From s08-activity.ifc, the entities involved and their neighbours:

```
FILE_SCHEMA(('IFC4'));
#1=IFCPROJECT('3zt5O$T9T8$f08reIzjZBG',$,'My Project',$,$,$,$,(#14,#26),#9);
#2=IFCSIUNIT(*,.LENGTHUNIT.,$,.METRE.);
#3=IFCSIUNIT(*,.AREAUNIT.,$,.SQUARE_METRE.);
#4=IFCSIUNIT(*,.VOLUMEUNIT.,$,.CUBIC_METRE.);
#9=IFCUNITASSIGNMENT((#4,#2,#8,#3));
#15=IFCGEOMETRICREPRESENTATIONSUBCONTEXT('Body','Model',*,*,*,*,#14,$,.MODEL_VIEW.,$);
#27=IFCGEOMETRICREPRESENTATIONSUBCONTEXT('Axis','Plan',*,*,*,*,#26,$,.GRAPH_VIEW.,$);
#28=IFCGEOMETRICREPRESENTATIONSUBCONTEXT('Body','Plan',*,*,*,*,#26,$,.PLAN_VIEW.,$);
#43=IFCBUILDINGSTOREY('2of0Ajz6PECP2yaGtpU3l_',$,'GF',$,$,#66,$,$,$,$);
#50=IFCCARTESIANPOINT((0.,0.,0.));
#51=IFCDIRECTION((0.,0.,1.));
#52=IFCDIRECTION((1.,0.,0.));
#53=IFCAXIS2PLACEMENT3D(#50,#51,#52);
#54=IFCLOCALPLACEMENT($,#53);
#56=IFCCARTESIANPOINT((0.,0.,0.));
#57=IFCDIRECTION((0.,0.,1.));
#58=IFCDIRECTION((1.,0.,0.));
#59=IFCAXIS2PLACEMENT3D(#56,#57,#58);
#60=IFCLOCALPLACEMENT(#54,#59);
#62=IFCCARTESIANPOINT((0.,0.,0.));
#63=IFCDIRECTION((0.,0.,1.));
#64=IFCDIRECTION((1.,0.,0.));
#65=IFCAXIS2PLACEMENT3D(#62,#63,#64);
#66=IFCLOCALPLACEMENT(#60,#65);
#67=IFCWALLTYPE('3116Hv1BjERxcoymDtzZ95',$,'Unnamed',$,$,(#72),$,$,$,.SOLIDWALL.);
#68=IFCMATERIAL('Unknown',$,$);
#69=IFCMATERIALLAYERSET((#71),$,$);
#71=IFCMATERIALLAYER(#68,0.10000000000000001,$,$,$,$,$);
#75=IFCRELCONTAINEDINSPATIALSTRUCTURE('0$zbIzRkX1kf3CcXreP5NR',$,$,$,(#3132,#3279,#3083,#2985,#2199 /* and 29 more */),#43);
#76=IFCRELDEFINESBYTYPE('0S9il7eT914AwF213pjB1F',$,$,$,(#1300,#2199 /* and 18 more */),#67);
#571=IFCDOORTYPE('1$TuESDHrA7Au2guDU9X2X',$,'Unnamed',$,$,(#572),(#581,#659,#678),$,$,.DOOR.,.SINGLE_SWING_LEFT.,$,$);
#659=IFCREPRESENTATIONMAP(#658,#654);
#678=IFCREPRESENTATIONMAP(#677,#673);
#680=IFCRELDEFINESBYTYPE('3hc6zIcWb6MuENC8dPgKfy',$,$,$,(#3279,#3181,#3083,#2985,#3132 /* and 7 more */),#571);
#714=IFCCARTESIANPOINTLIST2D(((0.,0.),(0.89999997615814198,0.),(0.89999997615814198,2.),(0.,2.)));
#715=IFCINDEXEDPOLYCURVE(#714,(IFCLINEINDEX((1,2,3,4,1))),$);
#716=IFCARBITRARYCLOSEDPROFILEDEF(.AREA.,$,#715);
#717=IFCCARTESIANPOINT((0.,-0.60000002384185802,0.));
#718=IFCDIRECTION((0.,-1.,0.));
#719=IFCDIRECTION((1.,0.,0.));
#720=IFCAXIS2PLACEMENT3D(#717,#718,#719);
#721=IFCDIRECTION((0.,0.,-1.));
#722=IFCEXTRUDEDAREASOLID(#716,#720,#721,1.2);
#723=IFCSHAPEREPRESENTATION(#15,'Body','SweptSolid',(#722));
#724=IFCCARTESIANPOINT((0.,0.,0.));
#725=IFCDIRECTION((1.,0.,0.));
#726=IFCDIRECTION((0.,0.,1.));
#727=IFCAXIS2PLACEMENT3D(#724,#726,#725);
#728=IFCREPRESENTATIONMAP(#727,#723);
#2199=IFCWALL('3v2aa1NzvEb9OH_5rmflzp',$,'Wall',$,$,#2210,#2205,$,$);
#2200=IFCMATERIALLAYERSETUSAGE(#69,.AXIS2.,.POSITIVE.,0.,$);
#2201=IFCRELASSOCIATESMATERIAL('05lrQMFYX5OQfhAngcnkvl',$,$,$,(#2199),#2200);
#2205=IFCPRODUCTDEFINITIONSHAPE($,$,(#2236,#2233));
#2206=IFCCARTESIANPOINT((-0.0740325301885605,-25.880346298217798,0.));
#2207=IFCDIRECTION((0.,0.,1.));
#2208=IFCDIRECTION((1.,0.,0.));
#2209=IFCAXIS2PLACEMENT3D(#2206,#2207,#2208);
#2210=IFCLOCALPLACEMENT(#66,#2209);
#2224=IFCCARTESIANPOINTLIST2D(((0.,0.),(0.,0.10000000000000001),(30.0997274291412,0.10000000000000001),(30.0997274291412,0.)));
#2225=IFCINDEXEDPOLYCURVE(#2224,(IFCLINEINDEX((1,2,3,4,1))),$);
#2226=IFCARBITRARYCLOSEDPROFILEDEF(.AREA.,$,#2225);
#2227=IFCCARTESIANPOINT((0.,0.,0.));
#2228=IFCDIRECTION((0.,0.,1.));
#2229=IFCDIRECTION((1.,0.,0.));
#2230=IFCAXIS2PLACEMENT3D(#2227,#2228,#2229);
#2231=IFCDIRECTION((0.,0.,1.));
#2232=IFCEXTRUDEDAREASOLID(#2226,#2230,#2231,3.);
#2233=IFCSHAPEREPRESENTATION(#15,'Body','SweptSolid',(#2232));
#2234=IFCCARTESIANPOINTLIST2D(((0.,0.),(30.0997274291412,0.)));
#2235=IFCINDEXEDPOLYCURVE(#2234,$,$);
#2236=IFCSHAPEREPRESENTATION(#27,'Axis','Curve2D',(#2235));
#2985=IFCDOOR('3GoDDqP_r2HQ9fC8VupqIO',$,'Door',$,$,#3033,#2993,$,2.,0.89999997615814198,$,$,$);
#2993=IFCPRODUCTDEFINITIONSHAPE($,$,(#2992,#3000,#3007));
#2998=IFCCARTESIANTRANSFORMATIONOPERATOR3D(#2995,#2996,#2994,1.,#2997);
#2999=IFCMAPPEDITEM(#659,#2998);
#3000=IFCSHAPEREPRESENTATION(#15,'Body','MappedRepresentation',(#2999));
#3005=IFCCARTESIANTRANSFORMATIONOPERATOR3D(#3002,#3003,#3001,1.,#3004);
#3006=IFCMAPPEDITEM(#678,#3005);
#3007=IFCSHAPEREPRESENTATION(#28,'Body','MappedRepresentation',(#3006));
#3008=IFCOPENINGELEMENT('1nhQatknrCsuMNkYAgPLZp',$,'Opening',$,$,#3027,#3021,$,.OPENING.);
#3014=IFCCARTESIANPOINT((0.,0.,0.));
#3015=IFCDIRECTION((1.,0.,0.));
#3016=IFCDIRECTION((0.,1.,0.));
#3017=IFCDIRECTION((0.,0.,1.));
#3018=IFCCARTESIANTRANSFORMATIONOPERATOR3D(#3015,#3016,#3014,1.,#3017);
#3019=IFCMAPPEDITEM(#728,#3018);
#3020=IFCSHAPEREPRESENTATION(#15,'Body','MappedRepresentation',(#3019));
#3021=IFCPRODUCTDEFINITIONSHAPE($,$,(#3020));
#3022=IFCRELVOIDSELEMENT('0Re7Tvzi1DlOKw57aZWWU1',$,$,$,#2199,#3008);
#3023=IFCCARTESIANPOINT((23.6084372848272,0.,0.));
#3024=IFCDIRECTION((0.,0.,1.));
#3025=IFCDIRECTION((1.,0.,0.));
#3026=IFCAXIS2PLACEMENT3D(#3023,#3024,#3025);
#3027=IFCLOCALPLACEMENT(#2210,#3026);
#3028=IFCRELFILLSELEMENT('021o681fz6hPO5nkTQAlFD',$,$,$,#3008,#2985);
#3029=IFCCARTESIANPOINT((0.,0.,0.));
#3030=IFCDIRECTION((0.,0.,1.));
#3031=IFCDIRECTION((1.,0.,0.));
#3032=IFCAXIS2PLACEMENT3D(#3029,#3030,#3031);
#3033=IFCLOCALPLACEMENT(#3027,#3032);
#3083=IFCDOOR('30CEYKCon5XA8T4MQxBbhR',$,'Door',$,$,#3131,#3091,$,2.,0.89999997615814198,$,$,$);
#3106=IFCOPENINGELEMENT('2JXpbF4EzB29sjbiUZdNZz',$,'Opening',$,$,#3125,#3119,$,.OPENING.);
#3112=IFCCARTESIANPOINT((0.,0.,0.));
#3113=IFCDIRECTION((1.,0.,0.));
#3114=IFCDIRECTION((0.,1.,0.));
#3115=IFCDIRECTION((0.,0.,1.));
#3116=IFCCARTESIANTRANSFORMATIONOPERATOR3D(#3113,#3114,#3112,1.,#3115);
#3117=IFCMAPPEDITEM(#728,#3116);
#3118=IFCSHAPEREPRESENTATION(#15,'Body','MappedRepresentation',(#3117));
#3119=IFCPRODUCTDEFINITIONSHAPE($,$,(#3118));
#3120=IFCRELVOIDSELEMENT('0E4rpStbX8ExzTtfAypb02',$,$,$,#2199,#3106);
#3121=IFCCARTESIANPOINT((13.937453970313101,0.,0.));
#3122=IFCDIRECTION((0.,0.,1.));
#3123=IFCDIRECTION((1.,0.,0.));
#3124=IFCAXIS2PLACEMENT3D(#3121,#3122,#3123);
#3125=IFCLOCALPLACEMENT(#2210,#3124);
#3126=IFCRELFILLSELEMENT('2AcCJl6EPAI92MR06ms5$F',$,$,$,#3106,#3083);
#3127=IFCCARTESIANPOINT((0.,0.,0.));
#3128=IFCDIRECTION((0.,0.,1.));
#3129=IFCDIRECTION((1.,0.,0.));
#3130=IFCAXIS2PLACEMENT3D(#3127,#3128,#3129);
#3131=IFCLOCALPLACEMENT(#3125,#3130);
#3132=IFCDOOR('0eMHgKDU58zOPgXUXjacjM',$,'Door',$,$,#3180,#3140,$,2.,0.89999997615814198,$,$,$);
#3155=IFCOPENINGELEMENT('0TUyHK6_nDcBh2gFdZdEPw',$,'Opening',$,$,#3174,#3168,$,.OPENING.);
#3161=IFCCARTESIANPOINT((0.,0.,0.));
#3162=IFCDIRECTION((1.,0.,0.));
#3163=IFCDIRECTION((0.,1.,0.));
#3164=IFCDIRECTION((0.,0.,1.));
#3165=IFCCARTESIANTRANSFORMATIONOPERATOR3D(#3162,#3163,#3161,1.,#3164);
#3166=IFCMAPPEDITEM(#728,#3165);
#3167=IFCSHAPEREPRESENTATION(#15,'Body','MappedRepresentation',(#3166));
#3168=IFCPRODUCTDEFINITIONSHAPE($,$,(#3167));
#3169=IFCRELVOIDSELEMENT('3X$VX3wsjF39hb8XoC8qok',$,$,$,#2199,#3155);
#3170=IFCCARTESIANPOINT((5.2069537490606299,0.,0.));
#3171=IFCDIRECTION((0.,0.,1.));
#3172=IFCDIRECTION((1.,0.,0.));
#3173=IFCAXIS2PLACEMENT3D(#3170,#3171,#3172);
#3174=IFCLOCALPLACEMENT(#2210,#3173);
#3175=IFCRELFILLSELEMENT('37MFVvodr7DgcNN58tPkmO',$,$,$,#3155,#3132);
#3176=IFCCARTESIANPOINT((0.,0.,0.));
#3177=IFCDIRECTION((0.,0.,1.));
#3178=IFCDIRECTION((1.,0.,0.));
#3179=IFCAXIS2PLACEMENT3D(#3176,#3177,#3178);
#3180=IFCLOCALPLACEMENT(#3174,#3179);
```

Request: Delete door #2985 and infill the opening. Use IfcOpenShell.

```python
import ifcopenshell
import ifcopenshell.api.feature
import ifcopenshell.api.root
import ifcopenshell.geom
import ifcopenshell.util.shape

model = ifcopenshell.open("s08-activity.ifc")
settings = ifcopenshell.geom.settings()


def volume(element):
    """Net volume in cubic metres, openings subtracted."""
    shape = ifcopenshell.geom.create_shape(settings, element)
    return ifcopenshell.util.shape.get_volume(shape.geometry)


door = model.by_guid("3GoDDqP_r2HQ9fC8VupqIO")
opening = door.FillsVoids[0].RelatingOpeningElement
wall = opening.VoidsElements[0].RelatingBuildingElement
before = volume(wall)

ifcopenshell.api.root.remove_product(model, product=door)
ifcopenshell.api.feature.remove_feature(model, feature=opening)

after = volume(wall)

print(f"wall volume {before:.3f} -> {after:.3f} m3")

model.write("s08-activity_rev.ifc")
```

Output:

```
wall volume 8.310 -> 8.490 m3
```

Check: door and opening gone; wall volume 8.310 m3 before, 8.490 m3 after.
